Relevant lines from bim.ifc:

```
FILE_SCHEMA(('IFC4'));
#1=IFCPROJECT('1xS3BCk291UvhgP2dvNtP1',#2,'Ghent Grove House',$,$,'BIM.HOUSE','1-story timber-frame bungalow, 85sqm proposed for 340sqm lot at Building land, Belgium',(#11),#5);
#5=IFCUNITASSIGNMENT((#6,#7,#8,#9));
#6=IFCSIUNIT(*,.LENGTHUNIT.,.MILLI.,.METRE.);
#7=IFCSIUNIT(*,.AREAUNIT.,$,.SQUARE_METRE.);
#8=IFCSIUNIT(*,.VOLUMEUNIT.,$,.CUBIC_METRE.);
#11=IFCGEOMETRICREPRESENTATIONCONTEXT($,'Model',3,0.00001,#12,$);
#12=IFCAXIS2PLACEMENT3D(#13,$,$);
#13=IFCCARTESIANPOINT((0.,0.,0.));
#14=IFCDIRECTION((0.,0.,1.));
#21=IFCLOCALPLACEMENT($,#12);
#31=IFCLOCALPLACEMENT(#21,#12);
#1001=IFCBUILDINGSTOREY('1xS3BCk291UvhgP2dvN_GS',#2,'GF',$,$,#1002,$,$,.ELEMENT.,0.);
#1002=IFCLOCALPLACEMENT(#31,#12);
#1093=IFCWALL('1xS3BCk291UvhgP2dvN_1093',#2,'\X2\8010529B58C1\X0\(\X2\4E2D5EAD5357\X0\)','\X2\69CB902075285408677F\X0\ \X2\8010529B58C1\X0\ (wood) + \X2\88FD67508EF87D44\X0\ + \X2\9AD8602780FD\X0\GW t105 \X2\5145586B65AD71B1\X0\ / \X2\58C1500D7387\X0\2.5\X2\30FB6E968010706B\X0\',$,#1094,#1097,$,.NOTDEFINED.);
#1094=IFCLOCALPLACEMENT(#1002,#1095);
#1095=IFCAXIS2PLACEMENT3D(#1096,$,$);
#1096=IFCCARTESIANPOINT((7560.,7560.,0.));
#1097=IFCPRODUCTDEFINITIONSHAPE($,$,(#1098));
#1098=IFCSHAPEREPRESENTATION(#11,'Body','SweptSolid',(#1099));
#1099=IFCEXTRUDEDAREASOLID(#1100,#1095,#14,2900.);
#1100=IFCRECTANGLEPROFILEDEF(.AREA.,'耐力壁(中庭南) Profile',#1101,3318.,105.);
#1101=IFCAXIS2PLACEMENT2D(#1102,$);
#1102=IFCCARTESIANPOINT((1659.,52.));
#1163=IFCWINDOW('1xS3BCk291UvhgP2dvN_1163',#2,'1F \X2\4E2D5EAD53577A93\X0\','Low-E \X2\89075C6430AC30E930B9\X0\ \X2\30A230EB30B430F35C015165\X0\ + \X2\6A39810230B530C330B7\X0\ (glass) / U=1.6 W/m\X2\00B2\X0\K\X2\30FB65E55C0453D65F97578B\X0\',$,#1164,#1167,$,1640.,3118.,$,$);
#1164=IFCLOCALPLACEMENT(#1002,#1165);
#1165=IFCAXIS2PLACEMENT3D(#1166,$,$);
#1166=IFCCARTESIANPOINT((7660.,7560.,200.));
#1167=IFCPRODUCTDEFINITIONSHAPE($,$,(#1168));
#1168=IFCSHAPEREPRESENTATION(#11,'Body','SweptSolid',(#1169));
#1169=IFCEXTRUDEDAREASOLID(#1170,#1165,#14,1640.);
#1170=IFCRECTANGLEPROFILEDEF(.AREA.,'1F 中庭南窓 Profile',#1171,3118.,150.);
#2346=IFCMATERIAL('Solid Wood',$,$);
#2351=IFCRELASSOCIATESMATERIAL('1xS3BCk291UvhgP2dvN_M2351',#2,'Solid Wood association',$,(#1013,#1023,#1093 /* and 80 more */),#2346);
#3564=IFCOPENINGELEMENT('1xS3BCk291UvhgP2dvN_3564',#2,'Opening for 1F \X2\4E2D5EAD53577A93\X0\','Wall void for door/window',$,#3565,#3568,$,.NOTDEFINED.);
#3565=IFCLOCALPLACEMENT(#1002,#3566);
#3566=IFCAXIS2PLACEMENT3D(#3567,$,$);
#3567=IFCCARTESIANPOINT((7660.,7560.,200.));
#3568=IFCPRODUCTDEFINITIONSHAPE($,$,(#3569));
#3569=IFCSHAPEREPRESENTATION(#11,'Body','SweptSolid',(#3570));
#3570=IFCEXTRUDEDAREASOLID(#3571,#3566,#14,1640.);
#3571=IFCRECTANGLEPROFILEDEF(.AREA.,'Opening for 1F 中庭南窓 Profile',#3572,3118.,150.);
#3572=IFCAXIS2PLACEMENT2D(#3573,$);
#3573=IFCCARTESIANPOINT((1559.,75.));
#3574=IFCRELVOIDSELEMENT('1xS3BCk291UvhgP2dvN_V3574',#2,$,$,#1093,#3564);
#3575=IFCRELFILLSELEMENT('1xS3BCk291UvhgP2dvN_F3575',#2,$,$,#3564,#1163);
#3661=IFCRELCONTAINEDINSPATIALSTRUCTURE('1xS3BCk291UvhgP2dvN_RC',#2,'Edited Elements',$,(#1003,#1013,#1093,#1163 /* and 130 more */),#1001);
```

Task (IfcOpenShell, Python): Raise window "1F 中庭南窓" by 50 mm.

```python
import numpy as np
import ifcopenshell
import ifcopenshell.api.geometry
import ifcopenshell.util.placement
import ifcopenshell.util.unit

model = ifcopenshell.open("bim.ifc")
unit_scale = ifcopenshell.util.unit.calculate_unit_scale(model)

window = model.by_guid("1xS3BCk291UvhgP2dvN_1163")
opening = window.FillsVoids[0].RelatingOpeningElement
dz = 50.0

shift = np.array([0.0, 0.0, dz])
# The window is not placed relative to its opening, so move both.
for product in (opening, window):
    matrix = ifcopenshell.util.placement.get_local_placement(product.ObjectPlacement)
    matrix[:3, 3] += shift
    ifcopenshell.api.geometry.edit_object_placement(model, product=product, matrix=matrix, is_si=False)

print(f"moved by {dz * unit_scale:+.3f} m")

model.write("bim_v2.ifc")
```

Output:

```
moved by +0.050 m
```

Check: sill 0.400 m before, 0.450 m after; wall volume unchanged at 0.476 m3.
